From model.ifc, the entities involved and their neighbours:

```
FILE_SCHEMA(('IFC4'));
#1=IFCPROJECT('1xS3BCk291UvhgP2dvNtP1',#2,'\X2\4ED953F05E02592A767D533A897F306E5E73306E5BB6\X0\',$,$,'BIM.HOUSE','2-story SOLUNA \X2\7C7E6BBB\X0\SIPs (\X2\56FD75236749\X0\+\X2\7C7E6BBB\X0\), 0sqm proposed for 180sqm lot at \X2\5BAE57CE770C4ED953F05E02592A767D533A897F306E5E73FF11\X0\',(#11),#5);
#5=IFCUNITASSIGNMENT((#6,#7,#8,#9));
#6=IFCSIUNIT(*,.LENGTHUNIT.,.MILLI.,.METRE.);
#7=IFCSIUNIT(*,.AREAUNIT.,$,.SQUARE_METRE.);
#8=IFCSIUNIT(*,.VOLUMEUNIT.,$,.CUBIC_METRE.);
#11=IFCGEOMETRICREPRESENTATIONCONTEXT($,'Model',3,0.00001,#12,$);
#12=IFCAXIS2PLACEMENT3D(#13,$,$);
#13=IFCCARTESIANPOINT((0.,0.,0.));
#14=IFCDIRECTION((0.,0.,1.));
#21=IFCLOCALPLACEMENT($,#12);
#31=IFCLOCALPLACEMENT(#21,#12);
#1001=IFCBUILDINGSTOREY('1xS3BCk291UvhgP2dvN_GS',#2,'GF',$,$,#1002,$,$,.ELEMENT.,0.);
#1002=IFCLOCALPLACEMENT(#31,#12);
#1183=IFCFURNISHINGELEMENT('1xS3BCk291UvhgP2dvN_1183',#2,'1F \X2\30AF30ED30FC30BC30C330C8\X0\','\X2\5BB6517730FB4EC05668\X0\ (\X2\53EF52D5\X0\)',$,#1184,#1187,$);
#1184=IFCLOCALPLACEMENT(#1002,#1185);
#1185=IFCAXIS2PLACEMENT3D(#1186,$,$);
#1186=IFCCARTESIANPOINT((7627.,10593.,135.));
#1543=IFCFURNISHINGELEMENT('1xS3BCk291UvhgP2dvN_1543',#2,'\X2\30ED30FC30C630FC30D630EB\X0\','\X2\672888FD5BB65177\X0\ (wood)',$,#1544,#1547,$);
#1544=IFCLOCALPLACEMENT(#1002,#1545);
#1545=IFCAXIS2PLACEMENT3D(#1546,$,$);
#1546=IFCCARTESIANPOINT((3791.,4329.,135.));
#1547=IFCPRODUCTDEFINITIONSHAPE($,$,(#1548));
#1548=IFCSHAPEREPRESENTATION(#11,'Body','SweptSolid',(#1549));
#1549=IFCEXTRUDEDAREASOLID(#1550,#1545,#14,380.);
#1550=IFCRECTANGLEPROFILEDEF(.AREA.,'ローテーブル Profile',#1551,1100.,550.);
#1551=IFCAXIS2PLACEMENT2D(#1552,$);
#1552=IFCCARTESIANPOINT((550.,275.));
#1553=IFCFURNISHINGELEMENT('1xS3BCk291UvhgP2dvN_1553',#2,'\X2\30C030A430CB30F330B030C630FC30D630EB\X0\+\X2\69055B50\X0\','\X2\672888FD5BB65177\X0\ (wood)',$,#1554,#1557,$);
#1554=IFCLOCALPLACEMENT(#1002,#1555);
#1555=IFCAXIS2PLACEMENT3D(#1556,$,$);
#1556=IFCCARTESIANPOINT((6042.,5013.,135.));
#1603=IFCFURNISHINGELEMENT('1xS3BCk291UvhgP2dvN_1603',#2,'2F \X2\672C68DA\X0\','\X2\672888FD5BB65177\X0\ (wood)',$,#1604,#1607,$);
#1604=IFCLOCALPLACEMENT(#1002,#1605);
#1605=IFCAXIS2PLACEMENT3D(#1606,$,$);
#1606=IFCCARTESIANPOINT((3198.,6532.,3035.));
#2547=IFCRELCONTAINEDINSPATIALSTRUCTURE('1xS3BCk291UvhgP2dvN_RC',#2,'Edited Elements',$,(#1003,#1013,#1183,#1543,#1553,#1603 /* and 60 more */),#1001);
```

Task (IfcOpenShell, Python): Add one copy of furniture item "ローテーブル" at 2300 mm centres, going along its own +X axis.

```python
import ifcopenshell
import ifcopenshell.api.geometry
import ifcopenshell.api.root
import ifcopenshell.util.element
import ifcopenshell.util.placement
import ifcopenshell.util.unit

model = ifcopenshell.open("model.ifc")
unit_scale = ifcopenshell.util.unit.calculate_unit_scale(model)


def reuse_history(source, copy):
    """copy_class also copies each property set's owner history, people and application; keep the originals."""
    for rel in copy.IsDefinedBy:
        if rel.is_a("IfcRelDefinesByProperties") and (history := rel.RelatingPropertyDefinition.OwnerHistory):
            rel.RelatingPropertyDefinition.OwnerHistory = source.OwnerHistory
            ifcopenshell.util.element.remove_deep2(model, history)


source = model.by_guid("1xS3BCk291UvhgP2dvN_1543")
base = ifcopenshell.util.placement.get_local_placement(source.ObjectPlacement)
step = base[:3, 0] * 2.3 / unit_scale

for i in range(1, 2):
    copy = ifcopenshell.api.root.copy_class(model, product=source)
    copy.Representation = ifcopenshell.util.element.copy_deep(
        model, source.Representation, exclude=["IfcGeometricRepresentationContext", "IfcRepresentationMap"]
    )
    reuse_history(source, copy)
    matrix = base.copy()
    matrix[:3, 3] += i * step
    print("added at", matrix[:3, 3].round(3) + 0.0)
    ifcopenshell.api.geometry.edit_object_placement(model, product=copy, matrix=matrix, is_si=False)

model.write("model_edited.ifc")
```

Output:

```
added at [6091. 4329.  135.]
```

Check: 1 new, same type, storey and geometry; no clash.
